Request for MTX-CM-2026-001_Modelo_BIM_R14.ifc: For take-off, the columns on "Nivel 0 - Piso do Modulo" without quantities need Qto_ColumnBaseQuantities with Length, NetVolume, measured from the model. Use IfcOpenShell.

First a look at what the model holds.

```python
import ifcopenshell
import ifcopenshell.util.element
import ifcopenshell.util.unit

model = ifcopenshell.open("MTX-CM-2026-001_Modelo_BIM_R14.ifc")
print(model.schema)
for unit_type in ("LENGTHUNIT", "AREAUNIT", "VOLUMEUNIT"):
    print(unit_type, ifcopenshell.util.unit.calculate_unit_scale(model, unit_type))
storey = next(s for s in model.by_type("IfcBuildingStorey") if s.Name == "Nivel 0 - Piso do Modulo")
columns = [e for e in ifcopenshell.util.element.get_decomposition(storey) if e.is_a("IfcColumn")]
for e in sorted(columns, key=lambda e: e.id()):
    print(e.id(), e.is_a(), e.Name, list(ifcopenshell.util.element.get_psets(e, qtos_only=True)), sep=" | ")
```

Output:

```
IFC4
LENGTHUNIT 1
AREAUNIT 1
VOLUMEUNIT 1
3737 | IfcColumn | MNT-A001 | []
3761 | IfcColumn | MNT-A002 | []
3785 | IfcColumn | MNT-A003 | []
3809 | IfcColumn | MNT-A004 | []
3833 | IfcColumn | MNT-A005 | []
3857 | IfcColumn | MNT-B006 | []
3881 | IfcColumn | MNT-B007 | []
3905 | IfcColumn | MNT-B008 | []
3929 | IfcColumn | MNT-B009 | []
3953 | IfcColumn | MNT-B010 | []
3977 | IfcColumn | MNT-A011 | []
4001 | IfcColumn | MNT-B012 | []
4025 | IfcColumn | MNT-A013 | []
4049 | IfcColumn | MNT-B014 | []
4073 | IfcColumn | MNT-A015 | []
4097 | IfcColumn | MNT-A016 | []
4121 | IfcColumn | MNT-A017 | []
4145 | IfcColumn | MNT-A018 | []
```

```python
import ifcopenshell
import ifcopenshell.api.pset
import ifcopenshell.geom
import ifcopenshell.util.element
import ifcopenshell.util.shape
import ifcopenshell.util.unit

model = ifcopenshell.open("MTX-CM-2026-001_Modelo_BIM_R14.ifc")
unit_scale = ifcopenshell.util.unit.calculate_unit_scale(model)
volume_scale = ifcopenshell.util.unit.calculate_unit_scale(model, "VOLUMEUNIT")
settings = ifcopenshell.geom.settings()

storey = next(s for s in model.by_type("IfcBuildingStorey") if s.Name == "Nivel 0 - Piso do Modulo")
columns = [e for e in ifcopenshell.util.element.get_decomposition(storey) if e.is_a("IfcColumn")]

for e in sorted(columns, key=lambda e: e.id()):
    if ifcopenshell.util.element.get_psets(e, qtos_only=True, should_inherit=False):
        continue
    # Geometry comes back in metres, in the element's own axes.
    shape = ifcopenshell.geom.create_shape(settings, e)
    values = {
        "Length": ifcopenshell.util.shape.get_z(shape.geometry) / unit_scale,
        "NetVolume": ifcopenshell.util.shape.get_volume(shape.geometry) / volume_scale,
    }
    qto = ifcopenshell.api.pset.add_qto(model, product=e, name="Qto_ColumnBaseQuantities")
    ifcopenshell.api.pset.edit_qto(model, qto=qto, properties=values)
    print(e.id(), {k: round(v, 3) for k, v in values.items()})

model.write("MTX-CM-2026-001_Modelo_BIM_R14_updated.ifc")
```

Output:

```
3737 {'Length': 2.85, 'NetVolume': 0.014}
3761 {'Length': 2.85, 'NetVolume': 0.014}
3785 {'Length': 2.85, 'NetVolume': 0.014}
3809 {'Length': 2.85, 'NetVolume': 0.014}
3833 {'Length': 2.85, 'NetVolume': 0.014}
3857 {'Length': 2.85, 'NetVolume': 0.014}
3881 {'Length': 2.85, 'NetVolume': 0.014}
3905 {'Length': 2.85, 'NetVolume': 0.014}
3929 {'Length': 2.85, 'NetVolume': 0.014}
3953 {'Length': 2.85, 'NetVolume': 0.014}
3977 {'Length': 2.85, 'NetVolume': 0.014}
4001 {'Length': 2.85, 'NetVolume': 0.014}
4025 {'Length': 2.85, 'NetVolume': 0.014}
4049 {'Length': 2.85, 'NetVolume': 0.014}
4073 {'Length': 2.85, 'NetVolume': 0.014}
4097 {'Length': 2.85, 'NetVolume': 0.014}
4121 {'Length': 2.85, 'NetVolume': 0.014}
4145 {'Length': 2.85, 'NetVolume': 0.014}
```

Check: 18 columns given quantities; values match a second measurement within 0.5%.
